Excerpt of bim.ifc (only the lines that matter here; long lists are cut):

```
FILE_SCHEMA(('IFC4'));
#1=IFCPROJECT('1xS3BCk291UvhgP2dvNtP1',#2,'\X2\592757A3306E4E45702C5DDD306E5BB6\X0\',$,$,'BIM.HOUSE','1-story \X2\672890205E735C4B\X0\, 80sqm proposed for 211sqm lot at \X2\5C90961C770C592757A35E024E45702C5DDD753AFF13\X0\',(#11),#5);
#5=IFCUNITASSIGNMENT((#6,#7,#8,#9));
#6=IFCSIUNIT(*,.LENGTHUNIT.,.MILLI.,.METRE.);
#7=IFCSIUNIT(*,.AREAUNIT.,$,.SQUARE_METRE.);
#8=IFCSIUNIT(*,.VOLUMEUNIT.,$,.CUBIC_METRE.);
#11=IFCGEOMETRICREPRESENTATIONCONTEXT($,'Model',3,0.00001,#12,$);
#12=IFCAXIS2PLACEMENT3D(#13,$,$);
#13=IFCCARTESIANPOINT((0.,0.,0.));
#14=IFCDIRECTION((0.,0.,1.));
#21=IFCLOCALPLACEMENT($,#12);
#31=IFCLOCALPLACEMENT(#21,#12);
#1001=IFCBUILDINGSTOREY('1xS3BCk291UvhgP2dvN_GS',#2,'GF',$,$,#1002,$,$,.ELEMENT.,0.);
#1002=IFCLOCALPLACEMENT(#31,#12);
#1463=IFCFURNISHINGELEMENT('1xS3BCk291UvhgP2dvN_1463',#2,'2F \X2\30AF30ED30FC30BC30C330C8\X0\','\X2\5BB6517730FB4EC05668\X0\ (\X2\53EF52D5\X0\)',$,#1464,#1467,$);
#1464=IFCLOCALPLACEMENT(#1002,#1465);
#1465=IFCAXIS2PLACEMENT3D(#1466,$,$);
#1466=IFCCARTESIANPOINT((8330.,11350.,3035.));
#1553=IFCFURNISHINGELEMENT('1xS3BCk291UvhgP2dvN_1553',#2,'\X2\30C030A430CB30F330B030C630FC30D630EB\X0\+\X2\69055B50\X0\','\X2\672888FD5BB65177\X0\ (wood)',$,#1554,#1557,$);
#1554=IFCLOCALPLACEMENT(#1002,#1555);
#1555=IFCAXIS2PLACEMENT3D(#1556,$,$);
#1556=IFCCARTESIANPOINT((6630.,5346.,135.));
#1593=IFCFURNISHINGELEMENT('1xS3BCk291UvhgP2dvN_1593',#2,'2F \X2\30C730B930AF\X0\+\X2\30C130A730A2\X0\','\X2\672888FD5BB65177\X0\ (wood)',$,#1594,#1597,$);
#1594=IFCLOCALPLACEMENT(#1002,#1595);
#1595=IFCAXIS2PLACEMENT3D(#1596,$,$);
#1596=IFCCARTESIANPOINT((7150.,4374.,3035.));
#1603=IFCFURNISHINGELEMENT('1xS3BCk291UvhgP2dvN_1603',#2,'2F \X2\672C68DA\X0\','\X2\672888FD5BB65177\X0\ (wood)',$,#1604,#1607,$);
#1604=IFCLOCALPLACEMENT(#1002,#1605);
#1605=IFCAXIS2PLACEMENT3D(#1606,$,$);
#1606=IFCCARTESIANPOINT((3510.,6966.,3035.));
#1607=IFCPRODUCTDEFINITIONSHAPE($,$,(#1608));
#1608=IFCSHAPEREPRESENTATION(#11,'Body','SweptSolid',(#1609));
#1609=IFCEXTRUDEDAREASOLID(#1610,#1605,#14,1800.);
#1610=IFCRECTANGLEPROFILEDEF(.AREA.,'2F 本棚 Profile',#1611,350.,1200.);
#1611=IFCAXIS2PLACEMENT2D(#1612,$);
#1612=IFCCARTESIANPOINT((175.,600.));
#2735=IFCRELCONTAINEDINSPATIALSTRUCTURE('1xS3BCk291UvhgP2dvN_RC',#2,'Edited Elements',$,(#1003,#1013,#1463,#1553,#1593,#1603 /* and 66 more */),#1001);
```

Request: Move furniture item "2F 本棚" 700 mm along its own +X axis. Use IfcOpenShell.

```python
import ifcopenshell
import ifcopenshell.api.geometry
import ifcopenshell.util.placement

model = ifcopenshell.open("bim.ifc")

item = model.by_guid("1xS3BCk291UvhgP2dvN_1603")
matrix = ifcopenshell.util.placement.get_local_placement(item.ObjectPlacement)
matrix[:3, 3] += matrix[:3, 0] * 700.0
ifcopenshell.api.geometry.edit_object_placement(model, product=item, matrix=matrix, is_si=False)

print(ifcopenshell.util.placement.get_local_placement(item.ObjectPlacement).round(3) + 0.0)

model.write("bim-out.ifc")
```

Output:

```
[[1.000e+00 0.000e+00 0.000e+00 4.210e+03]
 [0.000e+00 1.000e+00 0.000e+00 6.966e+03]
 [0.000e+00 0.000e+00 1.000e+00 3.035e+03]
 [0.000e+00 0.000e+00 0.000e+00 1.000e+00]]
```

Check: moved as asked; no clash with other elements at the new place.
